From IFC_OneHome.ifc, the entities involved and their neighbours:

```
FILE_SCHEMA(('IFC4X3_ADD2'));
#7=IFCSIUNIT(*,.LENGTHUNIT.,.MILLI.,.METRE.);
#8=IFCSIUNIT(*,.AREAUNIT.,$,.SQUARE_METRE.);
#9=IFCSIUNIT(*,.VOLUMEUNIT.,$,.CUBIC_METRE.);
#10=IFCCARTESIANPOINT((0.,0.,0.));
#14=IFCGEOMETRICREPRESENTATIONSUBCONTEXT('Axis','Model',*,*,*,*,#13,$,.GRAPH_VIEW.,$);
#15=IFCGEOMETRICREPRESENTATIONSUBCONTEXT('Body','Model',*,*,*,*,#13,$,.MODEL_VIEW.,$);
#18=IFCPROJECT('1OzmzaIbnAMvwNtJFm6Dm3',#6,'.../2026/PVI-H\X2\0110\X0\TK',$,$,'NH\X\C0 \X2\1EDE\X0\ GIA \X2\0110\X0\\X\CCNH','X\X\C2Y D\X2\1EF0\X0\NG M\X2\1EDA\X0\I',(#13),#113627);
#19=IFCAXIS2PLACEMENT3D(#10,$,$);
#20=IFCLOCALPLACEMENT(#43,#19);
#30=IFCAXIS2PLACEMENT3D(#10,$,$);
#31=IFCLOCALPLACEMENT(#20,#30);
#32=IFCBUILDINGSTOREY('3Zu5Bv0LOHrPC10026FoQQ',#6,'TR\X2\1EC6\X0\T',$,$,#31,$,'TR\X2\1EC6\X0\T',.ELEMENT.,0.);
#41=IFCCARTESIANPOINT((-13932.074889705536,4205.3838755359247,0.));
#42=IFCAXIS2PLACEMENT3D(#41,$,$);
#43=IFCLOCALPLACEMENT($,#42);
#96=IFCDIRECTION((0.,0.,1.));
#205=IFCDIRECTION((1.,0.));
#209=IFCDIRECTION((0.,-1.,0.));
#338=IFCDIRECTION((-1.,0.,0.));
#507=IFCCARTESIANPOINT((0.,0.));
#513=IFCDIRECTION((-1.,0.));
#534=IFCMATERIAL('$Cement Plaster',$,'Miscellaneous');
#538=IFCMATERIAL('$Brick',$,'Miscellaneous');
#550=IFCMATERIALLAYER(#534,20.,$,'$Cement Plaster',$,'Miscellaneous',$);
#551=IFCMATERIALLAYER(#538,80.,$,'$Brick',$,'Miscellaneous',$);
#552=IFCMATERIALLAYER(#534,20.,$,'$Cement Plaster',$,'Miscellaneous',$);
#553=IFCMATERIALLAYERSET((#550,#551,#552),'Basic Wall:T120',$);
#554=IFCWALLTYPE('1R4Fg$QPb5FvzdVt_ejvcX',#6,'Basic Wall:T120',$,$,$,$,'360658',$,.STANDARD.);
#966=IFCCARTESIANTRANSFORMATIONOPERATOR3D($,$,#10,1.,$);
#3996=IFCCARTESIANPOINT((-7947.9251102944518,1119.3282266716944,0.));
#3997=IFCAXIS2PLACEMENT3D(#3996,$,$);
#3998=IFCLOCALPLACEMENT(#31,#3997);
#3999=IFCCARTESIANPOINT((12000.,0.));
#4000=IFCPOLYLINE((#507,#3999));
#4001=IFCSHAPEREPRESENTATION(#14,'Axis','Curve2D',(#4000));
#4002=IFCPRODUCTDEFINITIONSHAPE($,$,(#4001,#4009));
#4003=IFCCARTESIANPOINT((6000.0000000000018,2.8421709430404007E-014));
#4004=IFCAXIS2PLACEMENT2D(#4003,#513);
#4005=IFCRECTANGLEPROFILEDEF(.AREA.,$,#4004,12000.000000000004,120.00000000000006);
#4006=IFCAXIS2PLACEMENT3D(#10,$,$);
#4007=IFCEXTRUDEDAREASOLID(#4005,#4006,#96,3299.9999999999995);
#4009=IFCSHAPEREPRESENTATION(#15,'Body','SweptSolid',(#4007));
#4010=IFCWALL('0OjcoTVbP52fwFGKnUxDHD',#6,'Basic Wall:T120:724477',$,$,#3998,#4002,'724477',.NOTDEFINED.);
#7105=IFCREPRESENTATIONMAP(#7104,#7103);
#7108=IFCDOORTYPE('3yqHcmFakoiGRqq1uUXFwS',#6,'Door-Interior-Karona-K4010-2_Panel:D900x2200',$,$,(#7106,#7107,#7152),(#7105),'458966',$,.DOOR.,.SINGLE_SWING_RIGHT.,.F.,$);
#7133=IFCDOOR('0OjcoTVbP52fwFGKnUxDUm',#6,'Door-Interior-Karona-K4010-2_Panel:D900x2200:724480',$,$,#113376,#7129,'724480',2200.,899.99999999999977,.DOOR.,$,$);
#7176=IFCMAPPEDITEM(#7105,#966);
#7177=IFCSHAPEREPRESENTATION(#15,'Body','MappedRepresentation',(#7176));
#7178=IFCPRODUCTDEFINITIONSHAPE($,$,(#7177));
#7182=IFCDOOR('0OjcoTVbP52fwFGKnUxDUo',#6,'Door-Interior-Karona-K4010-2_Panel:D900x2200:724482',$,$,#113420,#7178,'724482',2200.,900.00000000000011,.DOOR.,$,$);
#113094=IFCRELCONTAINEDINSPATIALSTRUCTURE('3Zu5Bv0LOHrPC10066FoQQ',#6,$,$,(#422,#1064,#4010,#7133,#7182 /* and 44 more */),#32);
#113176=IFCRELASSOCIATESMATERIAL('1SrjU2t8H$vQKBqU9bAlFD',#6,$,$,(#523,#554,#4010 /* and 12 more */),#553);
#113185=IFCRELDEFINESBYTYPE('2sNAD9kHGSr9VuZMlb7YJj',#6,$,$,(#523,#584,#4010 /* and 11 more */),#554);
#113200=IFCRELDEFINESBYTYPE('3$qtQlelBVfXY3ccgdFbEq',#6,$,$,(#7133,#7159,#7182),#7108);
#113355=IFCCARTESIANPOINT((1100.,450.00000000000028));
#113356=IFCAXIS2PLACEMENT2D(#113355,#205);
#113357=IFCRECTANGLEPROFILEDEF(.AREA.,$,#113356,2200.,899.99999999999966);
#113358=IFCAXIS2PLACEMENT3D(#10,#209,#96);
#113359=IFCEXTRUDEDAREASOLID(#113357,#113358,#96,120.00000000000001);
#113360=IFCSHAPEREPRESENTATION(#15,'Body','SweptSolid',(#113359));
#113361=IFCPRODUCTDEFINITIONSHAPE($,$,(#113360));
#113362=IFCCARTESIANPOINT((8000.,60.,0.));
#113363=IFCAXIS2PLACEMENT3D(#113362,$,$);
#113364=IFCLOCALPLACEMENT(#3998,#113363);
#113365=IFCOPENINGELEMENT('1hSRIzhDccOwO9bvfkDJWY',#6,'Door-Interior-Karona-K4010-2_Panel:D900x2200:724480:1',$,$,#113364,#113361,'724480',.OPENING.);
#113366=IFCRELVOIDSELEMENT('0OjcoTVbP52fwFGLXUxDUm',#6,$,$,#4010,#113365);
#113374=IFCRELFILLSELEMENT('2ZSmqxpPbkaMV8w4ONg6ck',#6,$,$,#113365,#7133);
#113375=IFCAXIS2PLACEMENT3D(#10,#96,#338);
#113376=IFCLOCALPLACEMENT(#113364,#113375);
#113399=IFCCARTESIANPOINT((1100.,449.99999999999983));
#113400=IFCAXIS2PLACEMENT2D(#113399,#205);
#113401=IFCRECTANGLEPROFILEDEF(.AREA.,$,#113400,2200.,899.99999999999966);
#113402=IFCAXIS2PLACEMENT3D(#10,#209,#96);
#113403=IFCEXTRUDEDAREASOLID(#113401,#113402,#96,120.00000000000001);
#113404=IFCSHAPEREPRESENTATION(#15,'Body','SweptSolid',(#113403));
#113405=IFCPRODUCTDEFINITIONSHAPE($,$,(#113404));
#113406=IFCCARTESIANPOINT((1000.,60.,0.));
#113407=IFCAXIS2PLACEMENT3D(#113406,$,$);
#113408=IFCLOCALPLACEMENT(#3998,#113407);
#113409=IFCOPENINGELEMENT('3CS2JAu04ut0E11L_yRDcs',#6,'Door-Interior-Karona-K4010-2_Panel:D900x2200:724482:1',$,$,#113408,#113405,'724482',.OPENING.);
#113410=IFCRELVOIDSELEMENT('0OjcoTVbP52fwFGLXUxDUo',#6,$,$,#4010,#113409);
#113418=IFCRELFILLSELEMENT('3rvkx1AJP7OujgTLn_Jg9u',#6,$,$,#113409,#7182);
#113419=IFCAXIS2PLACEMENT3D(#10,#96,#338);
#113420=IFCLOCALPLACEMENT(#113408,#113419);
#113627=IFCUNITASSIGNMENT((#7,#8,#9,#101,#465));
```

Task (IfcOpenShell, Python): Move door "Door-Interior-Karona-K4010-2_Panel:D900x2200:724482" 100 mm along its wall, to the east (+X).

```python
import ifcopenshell
import ifcopenshell.api.geometry
import ifcopenshell.util.placement

model = ifcopenshell.open("IFC_OneHome.ifc")

door = model.by_guid("0OjcoTVbP52fwFGKnUxDUo")
opening = door.FillsVoids[0].RelatingOpeningElement
wall = opening.VoidsElements[0].RelatingBuildingElement

wall_matrix = ifcopenshell.util.placement.get_local_placement(wall.ObjectPlacement)
shift = wall_matrix[:3, 0] * 100.0
before = ifcopenshell.util.placement.get_local_placement(door.ObjectPlacement)[:3, 3].copy()

# The door is placed relative to its opening, so it follows when the opening moves.
matrix = ifcopenshell.util.placement.get_local_placement(opening.ObjectPlacement)
matrix[:3, 3] += shift
ifcopenshell.api.geometry.edit_object_placement(
    model, product=opening, matrix=matrix, is_si=False, should_transform_children=True
)

after = ifcopenshell.util.placement.get_local_placement(door.ObjectPlacement)[:3, 3]
print("door moved by", (after - before).round(3) + 0.0)

model.write("IFC_OneHome-out.ifc")
```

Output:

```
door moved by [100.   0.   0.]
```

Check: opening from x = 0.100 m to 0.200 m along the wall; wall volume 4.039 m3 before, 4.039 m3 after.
